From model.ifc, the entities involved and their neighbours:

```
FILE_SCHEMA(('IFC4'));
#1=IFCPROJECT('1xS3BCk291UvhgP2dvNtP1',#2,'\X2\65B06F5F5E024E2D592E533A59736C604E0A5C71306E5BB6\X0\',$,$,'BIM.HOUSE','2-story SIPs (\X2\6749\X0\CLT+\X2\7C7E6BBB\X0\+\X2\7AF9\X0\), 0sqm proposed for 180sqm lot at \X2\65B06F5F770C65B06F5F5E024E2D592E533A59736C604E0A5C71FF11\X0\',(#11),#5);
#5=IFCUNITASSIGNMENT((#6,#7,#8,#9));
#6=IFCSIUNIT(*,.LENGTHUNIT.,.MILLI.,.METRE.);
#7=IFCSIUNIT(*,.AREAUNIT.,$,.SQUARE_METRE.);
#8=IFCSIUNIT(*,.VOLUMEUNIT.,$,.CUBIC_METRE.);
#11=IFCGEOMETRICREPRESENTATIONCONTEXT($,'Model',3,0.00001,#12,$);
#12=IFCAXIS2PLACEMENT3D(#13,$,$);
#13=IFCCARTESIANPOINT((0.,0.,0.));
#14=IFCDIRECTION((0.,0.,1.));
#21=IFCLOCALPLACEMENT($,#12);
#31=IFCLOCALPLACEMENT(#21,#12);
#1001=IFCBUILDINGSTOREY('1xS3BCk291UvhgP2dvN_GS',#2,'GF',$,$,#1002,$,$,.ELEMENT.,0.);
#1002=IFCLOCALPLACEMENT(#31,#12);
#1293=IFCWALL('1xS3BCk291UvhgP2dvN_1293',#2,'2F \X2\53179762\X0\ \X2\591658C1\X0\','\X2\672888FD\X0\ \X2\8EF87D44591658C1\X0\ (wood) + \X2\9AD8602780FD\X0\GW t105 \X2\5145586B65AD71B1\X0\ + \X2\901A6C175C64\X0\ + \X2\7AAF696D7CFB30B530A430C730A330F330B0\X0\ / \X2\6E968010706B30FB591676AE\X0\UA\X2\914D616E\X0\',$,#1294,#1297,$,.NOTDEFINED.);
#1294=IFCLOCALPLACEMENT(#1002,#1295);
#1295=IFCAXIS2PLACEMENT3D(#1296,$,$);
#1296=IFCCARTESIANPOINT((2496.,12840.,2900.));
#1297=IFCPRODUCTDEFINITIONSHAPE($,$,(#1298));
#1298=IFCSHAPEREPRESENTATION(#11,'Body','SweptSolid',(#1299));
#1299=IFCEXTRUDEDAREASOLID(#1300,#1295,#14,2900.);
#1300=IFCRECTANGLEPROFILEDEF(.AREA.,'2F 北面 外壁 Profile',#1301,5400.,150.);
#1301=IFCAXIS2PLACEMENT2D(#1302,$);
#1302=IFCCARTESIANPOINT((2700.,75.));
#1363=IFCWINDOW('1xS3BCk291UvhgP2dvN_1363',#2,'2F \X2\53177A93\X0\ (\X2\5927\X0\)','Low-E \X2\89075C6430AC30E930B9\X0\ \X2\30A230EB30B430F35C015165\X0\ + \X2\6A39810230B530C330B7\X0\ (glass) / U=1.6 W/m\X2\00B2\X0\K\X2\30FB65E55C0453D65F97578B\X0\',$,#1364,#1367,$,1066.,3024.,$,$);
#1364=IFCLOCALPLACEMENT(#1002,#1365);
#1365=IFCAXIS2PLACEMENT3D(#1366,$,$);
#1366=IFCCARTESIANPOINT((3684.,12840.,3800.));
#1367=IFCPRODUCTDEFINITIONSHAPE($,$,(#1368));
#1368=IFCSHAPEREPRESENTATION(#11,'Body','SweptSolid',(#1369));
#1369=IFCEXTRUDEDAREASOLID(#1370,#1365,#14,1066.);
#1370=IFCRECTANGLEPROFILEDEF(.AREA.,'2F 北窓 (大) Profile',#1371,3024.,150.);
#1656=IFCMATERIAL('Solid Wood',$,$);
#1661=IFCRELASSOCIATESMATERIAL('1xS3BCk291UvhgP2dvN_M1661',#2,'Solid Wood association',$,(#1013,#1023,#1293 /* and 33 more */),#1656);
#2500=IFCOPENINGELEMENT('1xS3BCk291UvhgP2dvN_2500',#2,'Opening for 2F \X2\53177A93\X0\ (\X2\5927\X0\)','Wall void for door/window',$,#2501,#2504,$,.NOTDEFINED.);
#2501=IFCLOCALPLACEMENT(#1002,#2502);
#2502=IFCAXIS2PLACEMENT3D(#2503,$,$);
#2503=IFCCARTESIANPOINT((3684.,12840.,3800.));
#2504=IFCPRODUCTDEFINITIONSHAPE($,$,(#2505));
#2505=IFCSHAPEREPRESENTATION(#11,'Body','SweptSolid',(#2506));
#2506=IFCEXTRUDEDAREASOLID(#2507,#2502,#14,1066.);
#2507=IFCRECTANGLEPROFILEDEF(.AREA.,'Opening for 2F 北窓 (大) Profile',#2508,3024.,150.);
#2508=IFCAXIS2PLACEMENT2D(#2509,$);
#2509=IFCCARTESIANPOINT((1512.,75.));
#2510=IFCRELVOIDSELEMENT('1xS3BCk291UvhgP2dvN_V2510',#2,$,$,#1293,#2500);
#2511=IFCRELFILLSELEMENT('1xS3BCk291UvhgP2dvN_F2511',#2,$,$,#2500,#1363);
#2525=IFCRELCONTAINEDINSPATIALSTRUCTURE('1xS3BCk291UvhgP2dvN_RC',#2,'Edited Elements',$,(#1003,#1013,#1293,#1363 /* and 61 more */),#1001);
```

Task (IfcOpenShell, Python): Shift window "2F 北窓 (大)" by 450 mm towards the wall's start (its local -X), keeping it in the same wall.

```python
import ifcopenshell
import ifcopenshell.api.geometry
import ifcopenshell.util.placement

model = ifcopenshell.open("model.ifc")

window = model.by_guid("1xS3BCk291UvhgP2dvN_1363")
opening = window.FillsVoids[0].RelatingOpeningElement
wall = opening.VoidsElements[0].RelatingBuildingElement

wall_matrix = ifcopenshell.util.placement.get_local_placement(wall.ObjectPlacement)
shift = wall_matrix[:3, 0] * -450.0
before = ifcopenshell.util.placement.get_local_placement(window.ObjectPlacement)[:3, 3].copy()

# The window is not placed relative to its opening, so move both.
for product in (opening, window):
    matrix = ifcopenshell.util.placement.get_local_placement(product.ObjectPlacement)
    matrix[:3, 3] += shift
    ifcopenshell.api.geometry.edit_object_placement(model, product=product, matrix=matrix, is_si=False)

after = ifcopenshell.util.placement.get_local_placement(window.ObjectPlacement)[:3, 3]
print("window moved by", (after - before).round(3) + 0.0)

model.write("model-out.ifc")
```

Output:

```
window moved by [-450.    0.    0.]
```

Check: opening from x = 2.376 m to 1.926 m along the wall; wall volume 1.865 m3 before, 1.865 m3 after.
